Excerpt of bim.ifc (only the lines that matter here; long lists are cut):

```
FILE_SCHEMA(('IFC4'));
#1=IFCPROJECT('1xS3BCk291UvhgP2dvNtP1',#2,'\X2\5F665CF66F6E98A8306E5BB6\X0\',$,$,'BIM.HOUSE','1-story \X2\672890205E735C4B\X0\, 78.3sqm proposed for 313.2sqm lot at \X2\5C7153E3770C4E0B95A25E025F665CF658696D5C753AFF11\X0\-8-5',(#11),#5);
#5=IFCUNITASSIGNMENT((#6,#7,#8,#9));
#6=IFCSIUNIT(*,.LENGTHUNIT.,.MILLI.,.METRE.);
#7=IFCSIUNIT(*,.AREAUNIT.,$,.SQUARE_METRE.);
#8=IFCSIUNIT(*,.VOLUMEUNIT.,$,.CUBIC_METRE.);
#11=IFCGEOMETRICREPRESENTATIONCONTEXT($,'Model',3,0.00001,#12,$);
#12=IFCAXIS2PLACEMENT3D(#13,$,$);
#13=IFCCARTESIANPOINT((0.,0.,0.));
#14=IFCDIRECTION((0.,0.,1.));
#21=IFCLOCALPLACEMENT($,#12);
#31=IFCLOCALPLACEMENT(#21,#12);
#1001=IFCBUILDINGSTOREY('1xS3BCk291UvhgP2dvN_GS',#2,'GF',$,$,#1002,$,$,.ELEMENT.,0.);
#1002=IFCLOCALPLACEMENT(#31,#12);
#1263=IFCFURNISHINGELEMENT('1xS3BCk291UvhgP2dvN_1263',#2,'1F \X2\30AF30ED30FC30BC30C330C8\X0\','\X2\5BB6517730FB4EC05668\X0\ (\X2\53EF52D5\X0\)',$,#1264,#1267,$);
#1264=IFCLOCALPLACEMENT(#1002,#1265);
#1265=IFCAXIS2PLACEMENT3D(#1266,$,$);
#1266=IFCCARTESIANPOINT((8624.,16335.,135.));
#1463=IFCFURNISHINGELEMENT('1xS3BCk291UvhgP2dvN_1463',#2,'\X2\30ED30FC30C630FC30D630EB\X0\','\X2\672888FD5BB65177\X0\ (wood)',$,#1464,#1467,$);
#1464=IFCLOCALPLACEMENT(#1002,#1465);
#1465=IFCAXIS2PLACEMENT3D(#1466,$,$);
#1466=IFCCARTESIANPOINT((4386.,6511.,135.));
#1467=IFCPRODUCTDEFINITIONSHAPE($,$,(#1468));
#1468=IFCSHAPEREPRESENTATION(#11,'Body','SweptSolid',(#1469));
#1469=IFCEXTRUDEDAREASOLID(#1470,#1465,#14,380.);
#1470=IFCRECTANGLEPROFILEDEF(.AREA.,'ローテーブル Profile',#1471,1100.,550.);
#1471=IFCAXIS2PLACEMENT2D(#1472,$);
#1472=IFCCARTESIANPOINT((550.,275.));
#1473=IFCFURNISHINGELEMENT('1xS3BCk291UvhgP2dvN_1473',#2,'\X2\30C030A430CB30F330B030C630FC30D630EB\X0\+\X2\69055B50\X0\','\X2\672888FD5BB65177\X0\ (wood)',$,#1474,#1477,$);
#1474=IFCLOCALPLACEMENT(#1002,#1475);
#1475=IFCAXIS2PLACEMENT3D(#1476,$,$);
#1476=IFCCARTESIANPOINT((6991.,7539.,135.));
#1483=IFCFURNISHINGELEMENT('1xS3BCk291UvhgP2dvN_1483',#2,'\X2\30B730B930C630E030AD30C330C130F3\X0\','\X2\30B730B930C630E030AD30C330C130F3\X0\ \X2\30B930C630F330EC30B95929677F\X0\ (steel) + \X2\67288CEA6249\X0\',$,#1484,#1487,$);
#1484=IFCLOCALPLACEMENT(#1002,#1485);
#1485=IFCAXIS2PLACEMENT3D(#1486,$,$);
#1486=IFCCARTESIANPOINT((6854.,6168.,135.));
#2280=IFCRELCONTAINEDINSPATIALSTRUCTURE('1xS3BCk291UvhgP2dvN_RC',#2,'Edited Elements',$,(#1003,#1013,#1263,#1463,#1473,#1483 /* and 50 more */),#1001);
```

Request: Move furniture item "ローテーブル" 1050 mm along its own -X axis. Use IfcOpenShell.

```python
import ifcopenshell
import ifcopenshell.api.geometry
import ifcopenshell.util.placement

model = ifcopenshell.open("bim.ifc")

item = model.by_guid("1xS3BCk291UvhgP2dvN_1463")
matrix = ifcopenshell.util.placement.get_local_placement(item.ObjectPlacement)
matrix[:3, 3] -= matrix[:3, 0] * 1050.0
ifcopenshell.api.geometry.edit_object_placement(model, product=item, matrix=matrix, is_si=False)

print(ifcopenshell.util.placement.get_local_placement(item.ObjectPlacement).round(3) + 0.0)

model.write("bim_updated.ifc")
```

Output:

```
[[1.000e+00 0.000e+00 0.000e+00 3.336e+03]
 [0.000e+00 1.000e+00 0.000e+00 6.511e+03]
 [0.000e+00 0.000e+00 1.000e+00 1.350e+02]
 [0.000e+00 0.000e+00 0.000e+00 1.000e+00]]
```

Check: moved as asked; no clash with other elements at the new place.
